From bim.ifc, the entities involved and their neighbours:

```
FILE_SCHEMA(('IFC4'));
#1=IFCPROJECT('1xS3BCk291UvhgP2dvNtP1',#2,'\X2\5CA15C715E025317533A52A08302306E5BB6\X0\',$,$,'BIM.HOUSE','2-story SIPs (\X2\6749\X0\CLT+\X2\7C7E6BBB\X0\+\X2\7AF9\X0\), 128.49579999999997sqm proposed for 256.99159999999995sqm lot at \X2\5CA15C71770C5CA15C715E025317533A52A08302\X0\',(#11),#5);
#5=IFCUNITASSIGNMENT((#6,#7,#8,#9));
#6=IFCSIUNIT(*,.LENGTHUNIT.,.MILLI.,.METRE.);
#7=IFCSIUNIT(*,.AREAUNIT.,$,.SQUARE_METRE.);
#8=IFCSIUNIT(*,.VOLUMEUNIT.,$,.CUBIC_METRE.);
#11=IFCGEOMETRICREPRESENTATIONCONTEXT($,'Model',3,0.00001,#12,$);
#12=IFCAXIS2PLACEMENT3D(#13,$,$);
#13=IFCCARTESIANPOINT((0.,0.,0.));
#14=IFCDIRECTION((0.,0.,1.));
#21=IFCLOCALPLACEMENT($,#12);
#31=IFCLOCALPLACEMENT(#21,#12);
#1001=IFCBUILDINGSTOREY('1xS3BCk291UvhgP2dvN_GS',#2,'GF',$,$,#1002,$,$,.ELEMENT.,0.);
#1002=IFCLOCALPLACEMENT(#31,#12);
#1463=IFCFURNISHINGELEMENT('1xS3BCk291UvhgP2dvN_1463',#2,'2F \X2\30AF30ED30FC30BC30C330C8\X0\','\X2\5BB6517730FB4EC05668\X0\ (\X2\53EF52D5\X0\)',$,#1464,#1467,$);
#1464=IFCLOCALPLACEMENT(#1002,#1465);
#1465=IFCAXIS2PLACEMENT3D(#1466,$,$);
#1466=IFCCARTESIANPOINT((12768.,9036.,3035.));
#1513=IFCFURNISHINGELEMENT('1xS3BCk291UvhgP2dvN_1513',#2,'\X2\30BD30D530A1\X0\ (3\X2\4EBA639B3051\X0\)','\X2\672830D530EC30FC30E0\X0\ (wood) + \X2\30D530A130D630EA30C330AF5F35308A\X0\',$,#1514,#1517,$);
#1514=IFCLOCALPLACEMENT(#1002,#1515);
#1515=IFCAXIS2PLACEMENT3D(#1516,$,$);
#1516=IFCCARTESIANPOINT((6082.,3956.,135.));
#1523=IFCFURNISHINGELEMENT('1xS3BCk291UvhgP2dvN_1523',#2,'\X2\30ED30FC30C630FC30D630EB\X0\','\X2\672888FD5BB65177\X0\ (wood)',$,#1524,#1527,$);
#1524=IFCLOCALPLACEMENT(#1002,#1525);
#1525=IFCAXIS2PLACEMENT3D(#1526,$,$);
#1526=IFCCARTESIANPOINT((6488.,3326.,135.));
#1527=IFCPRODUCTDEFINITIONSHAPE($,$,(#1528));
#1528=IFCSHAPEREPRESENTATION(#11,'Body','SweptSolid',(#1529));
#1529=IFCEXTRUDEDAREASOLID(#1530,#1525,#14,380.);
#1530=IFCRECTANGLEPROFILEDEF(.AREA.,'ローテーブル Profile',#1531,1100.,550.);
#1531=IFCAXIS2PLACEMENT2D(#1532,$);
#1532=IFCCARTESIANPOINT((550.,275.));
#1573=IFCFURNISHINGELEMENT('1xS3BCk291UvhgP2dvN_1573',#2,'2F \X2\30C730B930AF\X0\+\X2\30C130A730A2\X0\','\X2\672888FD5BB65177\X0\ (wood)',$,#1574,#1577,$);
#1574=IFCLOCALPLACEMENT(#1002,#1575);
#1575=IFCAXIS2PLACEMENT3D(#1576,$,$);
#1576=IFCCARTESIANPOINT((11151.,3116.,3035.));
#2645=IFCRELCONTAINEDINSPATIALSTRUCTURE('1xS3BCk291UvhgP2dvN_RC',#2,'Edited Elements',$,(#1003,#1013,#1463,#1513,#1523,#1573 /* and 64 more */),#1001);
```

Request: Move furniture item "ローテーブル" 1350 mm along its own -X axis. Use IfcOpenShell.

```python
import ifcopenshell
import ifcopenshell.api.geometry
import ifcopenshell.util.placement
import ifcopenshell.util.unit

model = ifcopenshell.open("bim.ifc")
unit_scale = ifcopenshell.util.unit.calculate_unit_scale(model)

item = model.by_guid("1xS3BCk291UvhgP2dvN_1523")
matrix = ifcopenshell.util.placement.get_local_placement(item.ObjectPlacement)
matrix[:3, 3] -= matrix[:3, 0] * 1.35 / unit_scale
ifcopenshell.api.geometry.edit_object_placement(model, product=item, matrix=matrix, is_si=False)

print(ifcopenshell.util.placement.get_local_placement(item.ObjectPlacement).round(3) + 0.0)

model.write("bim_v2.ifc")
```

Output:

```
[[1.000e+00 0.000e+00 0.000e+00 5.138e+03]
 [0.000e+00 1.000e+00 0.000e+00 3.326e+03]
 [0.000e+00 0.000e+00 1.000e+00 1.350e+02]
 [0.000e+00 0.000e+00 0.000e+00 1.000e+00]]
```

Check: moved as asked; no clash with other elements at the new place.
